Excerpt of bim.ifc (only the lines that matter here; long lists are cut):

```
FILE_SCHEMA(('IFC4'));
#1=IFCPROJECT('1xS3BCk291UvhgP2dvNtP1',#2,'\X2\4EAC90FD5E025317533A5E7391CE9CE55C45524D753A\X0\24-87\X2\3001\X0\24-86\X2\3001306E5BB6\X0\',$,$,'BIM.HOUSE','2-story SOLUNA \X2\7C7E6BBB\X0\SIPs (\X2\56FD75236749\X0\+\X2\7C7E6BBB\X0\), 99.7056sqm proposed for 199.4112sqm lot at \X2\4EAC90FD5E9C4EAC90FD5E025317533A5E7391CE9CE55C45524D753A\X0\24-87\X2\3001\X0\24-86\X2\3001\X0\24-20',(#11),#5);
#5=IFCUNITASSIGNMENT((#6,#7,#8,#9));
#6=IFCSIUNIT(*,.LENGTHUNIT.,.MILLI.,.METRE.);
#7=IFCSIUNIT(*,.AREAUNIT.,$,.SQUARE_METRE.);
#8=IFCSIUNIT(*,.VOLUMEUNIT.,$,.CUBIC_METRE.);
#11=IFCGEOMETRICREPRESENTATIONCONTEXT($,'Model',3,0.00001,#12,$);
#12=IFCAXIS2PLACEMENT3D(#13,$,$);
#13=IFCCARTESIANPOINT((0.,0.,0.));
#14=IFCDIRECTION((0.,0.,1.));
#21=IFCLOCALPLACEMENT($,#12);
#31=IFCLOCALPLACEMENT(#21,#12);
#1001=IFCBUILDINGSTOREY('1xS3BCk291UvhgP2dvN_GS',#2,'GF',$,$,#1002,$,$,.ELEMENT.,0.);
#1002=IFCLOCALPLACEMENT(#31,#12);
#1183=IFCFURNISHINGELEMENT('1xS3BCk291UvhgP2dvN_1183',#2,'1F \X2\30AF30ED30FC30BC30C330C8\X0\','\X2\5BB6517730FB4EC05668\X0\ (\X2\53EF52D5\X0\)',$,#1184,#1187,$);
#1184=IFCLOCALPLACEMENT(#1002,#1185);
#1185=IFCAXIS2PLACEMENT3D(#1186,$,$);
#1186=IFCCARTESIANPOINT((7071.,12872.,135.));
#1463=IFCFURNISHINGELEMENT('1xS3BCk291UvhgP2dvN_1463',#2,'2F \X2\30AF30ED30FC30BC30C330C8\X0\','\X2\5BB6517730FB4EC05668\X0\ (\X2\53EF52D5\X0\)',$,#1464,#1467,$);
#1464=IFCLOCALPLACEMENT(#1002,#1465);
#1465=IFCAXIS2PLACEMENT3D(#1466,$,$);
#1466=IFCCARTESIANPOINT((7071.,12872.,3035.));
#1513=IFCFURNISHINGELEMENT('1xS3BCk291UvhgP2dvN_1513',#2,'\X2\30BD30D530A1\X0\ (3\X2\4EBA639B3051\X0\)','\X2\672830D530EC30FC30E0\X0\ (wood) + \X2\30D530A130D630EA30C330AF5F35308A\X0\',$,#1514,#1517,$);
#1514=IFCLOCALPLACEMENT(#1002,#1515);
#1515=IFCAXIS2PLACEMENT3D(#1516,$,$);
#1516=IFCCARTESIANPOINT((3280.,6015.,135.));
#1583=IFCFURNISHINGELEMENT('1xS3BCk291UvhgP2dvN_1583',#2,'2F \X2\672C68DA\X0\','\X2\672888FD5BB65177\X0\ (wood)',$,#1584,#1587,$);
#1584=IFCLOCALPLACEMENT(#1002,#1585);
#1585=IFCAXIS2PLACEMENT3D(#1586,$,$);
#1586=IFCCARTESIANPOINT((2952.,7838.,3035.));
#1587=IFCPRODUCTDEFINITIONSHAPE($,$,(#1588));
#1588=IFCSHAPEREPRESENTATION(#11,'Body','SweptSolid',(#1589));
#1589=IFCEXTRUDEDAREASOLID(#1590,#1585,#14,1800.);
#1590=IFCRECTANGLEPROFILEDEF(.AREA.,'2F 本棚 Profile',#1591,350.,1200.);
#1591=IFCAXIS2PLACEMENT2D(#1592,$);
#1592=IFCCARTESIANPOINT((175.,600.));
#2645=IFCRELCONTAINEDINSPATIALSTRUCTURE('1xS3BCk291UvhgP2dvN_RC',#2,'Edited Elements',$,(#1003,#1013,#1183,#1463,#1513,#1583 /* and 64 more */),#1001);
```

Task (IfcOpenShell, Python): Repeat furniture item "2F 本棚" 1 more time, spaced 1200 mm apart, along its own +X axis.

```python
import ifcopenshell
import ifcopenshell.api.geometry
import ifcopenshell.api.root
import ifcopenshell.util.element
import ifcopenshell.util.placement
import ifcopenshell.util.unit

model = ifcopenshell.open("bim.ifc")
unit_scale = ifcopenshell.util.unit.calculate_unit_scale(model)


def reuse_history(source, copy):
    """copy_class also copies each property set's owner history, people and application; keep the originals."""
    for rel in copy.IsDefinedBy:
        if rel.is_a("IfcRelDefinesByProperties") and (history := rel.RelatingPropertyDefinition.OwnerHistory):
            rel.RelatingPropertyDefinition.OwnerHistory = source.OwnerHistory
            ifcopenshell.util.element.remove_deep2(model, history)


source = model.by_id(1583)
base = ifcopenshell.util.placement.get_local_placement(source.ObjectPlacement)
step = base[:3, 0] * 1.2 / unit_scale

for i in range(1, 2):
    copy = ifcopenshell.api.root.copy_class(model, product=source)
    copy.Representation = ifcopenshell.util.element.copy_deep(
        model, source.Representation, exclude=["IfcGeometricRepresentationContext", "IfcRepresentationMap"]
    )
    reuse_history(source, copy)
    matrix = base.copy()
    matrix[:3, 3] += i * step
    print("added at", matrix[:3, 3].round(3) + 0.0)
    ifcopenshell.api.geometry.edit_object_placement(model, product=copy, matrix=matrix, is_si=False)

model.write("bim_updated.ifc")
```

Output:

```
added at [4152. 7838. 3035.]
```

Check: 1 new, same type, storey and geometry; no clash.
